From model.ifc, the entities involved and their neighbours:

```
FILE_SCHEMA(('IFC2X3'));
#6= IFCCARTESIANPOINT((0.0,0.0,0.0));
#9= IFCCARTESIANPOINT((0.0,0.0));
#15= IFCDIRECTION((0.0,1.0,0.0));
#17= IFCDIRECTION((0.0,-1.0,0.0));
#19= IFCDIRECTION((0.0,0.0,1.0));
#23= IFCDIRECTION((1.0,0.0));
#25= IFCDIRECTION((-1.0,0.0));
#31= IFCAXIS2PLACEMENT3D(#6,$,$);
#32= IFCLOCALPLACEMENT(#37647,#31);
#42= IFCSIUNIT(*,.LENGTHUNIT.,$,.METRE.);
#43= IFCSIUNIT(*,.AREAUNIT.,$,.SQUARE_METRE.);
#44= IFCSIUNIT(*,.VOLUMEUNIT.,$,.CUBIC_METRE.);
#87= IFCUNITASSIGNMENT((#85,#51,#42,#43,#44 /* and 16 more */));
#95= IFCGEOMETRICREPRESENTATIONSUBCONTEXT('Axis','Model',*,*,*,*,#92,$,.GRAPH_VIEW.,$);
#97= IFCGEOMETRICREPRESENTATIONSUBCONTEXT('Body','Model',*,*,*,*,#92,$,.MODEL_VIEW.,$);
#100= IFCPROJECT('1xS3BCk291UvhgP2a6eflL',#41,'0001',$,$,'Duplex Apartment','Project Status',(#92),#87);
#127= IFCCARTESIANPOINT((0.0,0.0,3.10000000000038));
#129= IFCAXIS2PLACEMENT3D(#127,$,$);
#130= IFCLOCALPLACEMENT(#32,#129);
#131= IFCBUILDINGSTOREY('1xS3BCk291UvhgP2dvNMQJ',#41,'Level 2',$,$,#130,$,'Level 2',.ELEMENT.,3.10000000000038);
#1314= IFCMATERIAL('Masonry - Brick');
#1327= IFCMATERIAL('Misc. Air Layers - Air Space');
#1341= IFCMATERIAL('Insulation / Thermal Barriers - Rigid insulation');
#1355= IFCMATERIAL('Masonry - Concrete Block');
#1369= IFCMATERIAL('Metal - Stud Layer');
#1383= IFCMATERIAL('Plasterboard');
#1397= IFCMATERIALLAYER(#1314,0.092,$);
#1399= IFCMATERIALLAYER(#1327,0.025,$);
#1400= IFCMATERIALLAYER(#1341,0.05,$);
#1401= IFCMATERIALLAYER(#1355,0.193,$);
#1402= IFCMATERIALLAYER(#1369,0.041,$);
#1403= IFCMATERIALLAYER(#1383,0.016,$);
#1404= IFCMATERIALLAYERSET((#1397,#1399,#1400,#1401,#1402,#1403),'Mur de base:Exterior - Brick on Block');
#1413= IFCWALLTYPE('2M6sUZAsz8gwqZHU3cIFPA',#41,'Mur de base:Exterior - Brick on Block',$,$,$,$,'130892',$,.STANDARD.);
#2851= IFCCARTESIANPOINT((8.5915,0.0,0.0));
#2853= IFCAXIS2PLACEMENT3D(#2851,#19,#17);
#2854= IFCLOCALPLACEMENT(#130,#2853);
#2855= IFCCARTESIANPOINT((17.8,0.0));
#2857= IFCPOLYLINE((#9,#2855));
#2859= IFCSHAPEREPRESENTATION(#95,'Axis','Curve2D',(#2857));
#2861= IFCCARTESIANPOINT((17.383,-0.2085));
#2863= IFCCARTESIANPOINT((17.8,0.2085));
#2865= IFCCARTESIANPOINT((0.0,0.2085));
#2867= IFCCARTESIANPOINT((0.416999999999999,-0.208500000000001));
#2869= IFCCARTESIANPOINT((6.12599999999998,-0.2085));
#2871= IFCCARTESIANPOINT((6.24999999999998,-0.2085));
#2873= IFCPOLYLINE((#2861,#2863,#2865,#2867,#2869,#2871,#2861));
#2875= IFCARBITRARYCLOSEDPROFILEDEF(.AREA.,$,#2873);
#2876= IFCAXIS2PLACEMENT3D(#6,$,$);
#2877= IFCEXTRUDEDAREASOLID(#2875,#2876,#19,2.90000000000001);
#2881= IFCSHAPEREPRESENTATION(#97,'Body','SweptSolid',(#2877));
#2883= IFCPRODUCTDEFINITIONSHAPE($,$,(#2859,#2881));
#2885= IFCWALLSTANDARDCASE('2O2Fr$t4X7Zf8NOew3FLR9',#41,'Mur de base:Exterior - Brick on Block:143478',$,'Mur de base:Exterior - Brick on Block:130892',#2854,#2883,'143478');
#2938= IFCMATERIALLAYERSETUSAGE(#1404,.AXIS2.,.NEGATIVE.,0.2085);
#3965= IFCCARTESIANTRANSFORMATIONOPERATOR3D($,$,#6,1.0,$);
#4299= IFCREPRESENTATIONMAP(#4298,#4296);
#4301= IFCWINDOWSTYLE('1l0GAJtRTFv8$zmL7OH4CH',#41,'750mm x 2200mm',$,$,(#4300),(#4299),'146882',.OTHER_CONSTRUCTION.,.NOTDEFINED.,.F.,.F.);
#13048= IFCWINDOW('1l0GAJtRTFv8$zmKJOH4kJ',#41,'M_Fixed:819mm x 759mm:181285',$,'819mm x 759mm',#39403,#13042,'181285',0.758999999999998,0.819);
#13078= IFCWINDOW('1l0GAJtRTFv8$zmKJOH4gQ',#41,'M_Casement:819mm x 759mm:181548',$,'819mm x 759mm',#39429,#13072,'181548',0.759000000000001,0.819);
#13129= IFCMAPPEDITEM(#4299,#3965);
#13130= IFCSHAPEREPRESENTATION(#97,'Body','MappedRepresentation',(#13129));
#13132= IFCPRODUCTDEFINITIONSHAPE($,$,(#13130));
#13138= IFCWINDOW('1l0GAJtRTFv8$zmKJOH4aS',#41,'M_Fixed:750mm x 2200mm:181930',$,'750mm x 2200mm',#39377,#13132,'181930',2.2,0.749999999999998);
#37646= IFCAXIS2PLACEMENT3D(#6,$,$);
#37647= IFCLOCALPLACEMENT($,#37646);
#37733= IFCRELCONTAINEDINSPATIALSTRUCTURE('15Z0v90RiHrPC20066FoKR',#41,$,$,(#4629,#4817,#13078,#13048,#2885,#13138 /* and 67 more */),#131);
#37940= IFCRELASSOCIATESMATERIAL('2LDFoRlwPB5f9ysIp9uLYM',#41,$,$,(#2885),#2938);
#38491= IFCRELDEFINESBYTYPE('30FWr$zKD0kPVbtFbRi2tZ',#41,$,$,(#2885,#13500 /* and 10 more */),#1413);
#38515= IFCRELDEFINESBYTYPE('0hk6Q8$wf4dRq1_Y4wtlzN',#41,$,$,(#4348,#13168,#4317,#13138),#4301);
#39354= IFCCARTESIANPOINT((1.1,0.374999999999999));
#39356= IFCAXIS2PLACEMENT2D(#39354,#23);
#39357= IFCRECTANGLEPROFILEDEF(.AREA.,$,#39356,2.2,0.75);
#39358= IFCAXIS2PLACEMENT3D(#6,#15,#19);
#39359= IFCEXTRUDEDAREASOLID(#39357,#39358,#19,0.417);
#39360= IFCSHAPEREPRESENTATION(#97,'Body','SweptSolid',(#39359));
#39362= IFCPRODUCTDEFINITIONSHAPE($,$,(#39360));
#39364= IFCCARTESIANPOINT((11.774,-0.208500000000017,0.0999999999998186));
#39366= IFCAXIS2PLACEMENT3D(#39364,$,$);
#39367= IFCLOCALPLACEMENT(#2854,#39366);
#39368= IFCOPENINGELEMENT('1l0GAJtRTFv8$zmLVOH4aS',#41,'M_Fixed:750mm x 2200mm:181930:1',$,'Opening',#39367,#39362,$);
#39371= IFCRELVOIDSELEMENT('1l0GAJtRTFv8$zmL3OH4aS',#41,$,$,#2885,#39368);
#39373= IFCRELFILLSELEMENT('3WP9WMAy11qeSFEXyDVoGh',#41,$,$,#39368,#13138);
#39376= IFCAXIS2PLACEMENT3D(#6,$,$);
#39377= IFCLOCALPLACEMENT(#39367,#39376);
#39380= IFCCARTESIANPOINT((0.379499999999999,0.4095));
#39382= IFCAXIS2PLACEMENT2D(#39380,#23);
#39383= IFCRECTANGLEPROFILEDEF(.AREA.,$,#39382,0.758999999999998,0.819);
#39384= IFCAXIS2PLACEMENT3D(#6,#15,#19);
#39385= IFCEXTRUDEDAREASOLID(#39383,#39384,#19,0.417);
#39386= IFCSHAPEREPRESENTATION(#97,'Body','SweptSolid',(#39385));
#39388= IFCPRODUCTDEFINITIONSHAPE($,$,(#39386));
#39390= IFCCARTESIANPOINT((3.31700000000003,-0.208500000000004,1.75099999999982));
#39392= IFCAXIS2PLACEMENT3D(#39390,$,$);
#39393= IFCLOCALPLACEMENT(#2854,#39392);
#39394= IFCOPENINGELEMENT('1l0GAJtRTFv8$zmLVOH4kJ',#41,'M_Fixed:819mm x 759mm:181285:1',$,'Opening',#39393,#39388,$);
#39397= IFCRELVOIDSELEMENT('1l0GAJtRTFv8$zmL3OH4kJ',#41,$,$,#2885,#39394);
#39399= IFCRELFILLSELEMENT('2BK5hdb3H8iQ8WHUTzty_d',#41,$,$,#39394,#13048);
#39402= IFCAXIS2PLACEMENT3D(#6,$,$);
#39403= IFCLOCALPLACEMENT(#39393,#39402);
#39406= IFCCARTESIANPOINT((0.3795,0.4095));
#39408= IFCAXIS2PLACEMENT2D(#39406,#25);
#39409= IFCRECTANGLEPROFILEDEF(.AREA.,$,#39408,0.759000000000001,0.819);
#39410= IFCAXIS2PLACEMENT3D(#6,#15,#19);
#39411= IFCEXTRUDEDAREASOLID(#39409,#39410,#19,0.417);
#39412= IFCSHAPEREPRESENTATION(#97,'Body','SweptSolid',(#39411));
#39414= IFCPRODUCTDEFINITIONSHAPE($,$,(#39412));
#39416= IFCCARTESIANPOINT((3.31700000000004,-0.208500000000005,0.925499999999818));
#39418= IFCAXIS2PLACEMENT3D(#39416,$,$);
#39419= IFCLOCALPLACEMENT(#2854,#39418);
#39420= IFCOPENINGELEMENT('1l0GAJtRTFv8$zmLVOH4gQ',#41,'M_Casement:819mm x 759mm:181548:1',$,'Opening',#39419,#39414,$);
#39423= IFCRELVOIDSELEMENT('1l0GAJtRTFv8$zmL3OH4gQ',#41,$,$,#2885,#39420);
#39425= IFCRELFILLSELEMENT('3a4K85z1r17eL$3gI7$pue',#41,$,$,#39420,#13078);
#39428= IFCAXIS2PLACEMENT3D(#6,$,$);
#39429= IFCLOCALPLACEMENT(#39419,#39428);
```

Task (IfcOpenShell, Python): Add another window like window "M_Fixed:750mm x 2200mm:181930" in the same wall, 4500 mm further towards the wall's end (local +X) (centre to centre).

```python
import ifcopenshell
import ifcopenshell.api.feature
import ifcopenshell.api.geometry
import ifcopenshell.api.root
import ifcopenshell.geom
import ifcopenshell.util.element
import ifcopenshell.util.placement
import ifcopenshell.util.shape
import ifcopenshell.util.unit

model = ifcopenshell.open("model.ifc")
unit_scale = ifcopenshell.util.unit.calculate_unit_scale(model)
settings = ifcopenshell.geom.settings()


def volume(element):
    """Net volume in cubic metres, openings subtracted."""
    shape = ifcopenshell.geom.create_shape(settings, element)
    return ifcopenshell.util.shape.get_volume(shape.geometry)


def reuse_history(source, copy):
    """copy_class also copies each property set's owner history, people and application; keep the originals."""
    for rel in copy.IsDefinedBy:
        if rel.is_a("IfcRelDefinesByProperties") and (history := rel.RelatingPropertyDefinition.OwnerHistory):
            rel.RelatingPropertyDefinition.OwnerHistory = source.OwnerHistory
            ifcopenshell.util.element.remove_deep2(model, history)


window = model.by_guid("1l0GAJtRTFv8$zmKJOH4aS")
opening = window.FillsVoids[0].RelatingOpeningElement
wall = opening.VoidsElements[0].RelatingBuildingElement
before = volume(wall)
shift = ifcopenshell.util.placement.get_local_placement(wall.ObjectPlacement)[:3, 0] * 4.5 / unit_scale

# copy_class copies the void relationship, type, container and properties, but no geometry.
new_opening = ifcopenshell.api.root.copy_class(model, product=opening)
new_opening.Representation = ifcopenshell.util.element.copy_deep(
    model, opening.Representation, exclude=["IfcGeometricRepresentationContext", "IfcRepresentationMap"]
)
new_opening.Name = "M_Fixed:750mm x 2200mm"
new_window = ifcopenshell.api.root.copy_class(model, product=window)
new_window.Representation = ifcopenshell.util.element.copy_deep(
    model, window.Representation, exclude=["IfcGeometricRepresentationContext", "IfcRepresentationMap"]
)
new_window.Name = "M_Fixed:750mm x 2200mm"
new_window.Tag = None
reuse_history(window, new_window)
fills = ifcopenshell.api.feature.add_filling(model, opening=new_opening, element=new_window)
fills.OwnerHistory = new_window.OwnerHistory  # required in IFC2X3

for old, new in ((opening, new_opening), (window, new_window)):
    matrix = ifcopenshell.util.placement.get_local_placement(old.ObjectPlacement)
    matrix[:3, 3] += shift
    ifcopenshell.api.geometry.edit_object_placement(model, product=new, matrix=matrix, is_si=False)

after = volume(wall)

print(f"wall volume {before:.3f} -> {after:.3f} m3")

model.write("model_rev.ifc")
```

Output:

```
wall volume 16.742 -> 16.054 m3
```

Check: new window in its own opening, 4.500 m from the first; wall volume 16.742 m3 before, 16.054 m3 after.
